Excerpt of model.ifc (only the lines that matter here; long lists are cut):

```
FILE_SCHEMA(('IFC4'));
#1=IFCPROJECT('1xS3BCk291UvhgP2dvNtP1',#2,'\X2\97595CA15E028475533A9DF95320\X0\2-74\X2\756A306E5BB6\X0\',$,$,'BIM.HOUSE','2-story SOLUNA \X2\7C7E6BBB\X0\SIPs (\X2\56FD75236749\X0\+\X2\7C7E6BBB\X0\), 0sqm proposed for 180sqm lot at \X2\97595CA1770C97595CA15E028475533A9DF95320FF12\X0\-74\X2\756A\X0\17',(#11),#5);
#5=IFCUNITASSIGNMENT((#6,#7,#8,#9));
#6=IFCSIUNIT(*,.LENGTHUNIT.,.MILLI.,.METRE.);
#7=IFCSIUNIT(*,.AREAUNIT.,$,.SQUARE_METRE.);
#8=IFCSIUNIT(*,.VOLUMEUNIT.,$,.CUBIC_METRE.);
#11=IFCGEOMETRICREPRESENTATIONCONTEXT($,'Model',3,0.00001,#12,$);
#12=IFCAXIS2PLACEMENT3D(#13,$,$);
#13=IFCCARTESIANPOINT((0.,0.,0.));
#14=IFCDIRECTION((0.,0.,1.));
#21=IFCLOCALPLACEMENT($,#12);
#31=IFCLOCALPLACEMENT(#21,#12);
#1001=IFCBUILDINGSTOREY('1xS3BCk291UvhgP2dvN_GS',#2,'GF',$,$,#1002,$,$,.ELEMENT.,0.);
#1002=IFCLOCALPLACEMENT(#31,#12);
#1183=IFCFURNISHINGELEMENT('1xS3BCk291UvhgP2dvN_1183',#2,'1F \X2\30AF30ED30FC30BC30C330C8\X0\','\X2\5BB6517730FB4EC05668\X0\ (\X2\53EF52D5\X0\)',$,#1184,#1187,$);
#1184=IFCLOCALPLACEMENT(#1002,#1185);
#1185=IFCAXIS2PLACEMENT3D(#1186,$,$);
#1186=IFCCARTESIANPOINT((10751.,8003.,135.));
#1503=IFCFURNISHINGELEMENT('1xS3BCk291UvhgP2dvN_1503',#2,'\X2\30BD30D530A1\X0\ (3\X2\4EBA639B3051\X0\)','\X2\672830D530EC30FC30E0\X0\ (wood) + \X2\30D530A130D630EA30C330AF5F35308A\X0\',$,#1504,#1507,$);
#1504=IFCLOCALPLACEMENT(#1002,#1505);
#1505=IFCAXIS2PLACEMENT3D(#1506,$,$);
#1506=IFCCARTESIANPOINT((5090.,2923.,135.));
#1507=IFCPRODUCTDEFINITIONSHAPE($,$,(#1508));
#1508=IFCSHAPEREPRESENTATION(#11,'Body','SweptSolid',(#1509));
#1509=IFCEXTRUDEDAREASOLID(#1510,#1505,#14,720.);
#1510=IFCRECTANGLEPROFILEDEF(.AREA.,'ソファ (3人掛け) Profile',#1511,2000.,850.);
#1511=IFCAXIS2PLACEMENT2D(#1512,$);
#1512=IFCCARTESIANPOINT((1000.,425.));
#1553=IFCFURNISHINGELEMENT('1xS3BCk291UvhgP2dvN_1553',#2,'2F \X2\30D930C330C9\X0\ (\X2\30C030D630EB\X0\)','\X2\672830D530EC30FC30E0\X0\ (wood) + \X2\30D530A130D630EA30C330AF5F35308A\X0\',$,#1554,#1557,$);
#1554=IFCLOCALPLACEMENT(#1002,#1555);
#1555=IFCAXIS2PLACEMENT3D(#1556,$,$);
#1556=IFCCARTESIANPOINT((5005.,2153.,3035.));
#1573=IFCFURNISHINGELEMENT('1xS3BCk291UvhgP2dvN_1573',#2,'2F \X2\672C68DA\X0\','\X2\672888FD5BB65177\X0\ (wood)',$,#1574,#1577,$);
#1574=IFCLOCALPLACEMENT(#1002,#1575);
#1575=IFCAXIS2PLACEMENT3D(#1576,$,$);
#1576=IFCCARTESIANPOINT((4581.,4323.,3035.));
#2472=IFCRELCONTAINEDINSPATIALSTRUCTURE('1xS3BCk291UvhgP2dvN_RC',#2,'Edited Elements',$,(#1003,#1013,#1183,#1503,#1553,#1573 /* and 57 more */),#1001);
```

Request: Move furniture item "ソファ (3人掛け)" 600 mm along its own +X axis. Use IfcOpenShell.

```python
import ifcopenshell
import ifcopenshell.api.geometry
import ifcopenshell.util.placement
import ifcopenshell.util.unit

model = ifcopenshell.open("model.ifc")
unit_scale = ifcopenshell.util.unit.calculate_unit_scale(model)

item = model.by_id(1503)
matrix = ifcopenshell.util.placement.get_local_placement(item.ObjectPlacement)
matrix[:3, 3] += matrix[:3, 0] * 0.6 / unit_scale
ifcopenshell.api.geometry.edit_object_placement(model, product=item, matrix=matrix, is_si=False)

print(ifcopenshell.util.placement.get_local_placement(item.ObjectPlacement).round(3) + 0.0)

model.write("model_updated.ifc")
```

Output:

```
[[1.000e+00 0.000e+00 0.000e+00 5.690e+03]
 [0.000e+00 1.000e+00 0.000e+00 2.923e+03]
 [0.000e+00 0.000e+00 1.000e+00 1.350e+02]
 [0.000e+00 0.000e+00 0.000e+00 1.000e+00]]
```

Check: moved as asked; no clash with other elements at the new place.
